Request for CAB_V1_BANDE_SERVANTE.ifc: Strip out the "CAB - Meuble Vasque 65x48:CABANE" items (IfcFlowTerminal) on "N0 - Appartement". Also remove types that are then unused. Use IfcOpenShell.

First a look at what the model holds.

```python
import ifcopenshell
import ifcopenshell.util.element

model = ifcopenshell.open("CAB_V1_BANDE_SERVANTE.ifc")
print(model.schema)
storey = next(s for s in model.by_type("IfcBuildingStorey") if s.Name == "N0 - Appartement")
terminals = [e for e in ifcopenshell.util.element.get_decomposition(storey) if e.is_a("IfcFlowTerminal")]
seen = {}
for e in terminals:
    element_type = ifcopenshell.util.element.get_type(e)
    name = element_type.Name if element_type not in (None, e) else None
    seen[name] = seen.get(name, 0) + 1
for name, count in sorted(seen.items(), key=str):
    print(count, "x", name)
```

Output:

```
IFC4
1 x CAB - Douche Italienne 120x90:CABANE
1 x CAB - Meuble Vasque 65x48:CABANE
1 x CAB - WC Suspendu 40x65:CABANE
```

```python
import ifcopenshell
import ifcopenshell.api.root
import ifcopenshell.util.element

model = ifcopenshell.open("CAB_V1_BANDE_SERVANTE.ifc")

storey = next(s for s in model.by_type("IfcBuildingStorey") if s.Name == "N0 - Appartement")
terminals = [e for e in ifcopenshell.util.element.get_decomposition(storey) if e.is_a("IfcFlowTerminal")]
targets = [e for e in terminals if (t := ifcopenshell.util.element.get_type(e)) not in (None, e) and t.Name == "CAB - Meuble Vasque 65x48:CABANE"]
types = {ifcopenshell.util.element.get_type(e) for e in targets} - {None, *targets}

for e in targets:
    ifcopenshell.api.root.remove_product(model, product=e)
print(len(targets), "removed")

unused = [t for t in types if not ifcopenshell.util.element.get_types(t)]
for t in unused:
    ifcopenshell.api.root.remove_product(model, product=t)
print(len(unused), "unused types removed")

model.write("CAB_V1_BANDE_SERVANTE_edited.ifc")
```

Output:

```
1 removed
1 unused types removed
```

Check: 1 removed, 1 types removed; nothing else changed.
